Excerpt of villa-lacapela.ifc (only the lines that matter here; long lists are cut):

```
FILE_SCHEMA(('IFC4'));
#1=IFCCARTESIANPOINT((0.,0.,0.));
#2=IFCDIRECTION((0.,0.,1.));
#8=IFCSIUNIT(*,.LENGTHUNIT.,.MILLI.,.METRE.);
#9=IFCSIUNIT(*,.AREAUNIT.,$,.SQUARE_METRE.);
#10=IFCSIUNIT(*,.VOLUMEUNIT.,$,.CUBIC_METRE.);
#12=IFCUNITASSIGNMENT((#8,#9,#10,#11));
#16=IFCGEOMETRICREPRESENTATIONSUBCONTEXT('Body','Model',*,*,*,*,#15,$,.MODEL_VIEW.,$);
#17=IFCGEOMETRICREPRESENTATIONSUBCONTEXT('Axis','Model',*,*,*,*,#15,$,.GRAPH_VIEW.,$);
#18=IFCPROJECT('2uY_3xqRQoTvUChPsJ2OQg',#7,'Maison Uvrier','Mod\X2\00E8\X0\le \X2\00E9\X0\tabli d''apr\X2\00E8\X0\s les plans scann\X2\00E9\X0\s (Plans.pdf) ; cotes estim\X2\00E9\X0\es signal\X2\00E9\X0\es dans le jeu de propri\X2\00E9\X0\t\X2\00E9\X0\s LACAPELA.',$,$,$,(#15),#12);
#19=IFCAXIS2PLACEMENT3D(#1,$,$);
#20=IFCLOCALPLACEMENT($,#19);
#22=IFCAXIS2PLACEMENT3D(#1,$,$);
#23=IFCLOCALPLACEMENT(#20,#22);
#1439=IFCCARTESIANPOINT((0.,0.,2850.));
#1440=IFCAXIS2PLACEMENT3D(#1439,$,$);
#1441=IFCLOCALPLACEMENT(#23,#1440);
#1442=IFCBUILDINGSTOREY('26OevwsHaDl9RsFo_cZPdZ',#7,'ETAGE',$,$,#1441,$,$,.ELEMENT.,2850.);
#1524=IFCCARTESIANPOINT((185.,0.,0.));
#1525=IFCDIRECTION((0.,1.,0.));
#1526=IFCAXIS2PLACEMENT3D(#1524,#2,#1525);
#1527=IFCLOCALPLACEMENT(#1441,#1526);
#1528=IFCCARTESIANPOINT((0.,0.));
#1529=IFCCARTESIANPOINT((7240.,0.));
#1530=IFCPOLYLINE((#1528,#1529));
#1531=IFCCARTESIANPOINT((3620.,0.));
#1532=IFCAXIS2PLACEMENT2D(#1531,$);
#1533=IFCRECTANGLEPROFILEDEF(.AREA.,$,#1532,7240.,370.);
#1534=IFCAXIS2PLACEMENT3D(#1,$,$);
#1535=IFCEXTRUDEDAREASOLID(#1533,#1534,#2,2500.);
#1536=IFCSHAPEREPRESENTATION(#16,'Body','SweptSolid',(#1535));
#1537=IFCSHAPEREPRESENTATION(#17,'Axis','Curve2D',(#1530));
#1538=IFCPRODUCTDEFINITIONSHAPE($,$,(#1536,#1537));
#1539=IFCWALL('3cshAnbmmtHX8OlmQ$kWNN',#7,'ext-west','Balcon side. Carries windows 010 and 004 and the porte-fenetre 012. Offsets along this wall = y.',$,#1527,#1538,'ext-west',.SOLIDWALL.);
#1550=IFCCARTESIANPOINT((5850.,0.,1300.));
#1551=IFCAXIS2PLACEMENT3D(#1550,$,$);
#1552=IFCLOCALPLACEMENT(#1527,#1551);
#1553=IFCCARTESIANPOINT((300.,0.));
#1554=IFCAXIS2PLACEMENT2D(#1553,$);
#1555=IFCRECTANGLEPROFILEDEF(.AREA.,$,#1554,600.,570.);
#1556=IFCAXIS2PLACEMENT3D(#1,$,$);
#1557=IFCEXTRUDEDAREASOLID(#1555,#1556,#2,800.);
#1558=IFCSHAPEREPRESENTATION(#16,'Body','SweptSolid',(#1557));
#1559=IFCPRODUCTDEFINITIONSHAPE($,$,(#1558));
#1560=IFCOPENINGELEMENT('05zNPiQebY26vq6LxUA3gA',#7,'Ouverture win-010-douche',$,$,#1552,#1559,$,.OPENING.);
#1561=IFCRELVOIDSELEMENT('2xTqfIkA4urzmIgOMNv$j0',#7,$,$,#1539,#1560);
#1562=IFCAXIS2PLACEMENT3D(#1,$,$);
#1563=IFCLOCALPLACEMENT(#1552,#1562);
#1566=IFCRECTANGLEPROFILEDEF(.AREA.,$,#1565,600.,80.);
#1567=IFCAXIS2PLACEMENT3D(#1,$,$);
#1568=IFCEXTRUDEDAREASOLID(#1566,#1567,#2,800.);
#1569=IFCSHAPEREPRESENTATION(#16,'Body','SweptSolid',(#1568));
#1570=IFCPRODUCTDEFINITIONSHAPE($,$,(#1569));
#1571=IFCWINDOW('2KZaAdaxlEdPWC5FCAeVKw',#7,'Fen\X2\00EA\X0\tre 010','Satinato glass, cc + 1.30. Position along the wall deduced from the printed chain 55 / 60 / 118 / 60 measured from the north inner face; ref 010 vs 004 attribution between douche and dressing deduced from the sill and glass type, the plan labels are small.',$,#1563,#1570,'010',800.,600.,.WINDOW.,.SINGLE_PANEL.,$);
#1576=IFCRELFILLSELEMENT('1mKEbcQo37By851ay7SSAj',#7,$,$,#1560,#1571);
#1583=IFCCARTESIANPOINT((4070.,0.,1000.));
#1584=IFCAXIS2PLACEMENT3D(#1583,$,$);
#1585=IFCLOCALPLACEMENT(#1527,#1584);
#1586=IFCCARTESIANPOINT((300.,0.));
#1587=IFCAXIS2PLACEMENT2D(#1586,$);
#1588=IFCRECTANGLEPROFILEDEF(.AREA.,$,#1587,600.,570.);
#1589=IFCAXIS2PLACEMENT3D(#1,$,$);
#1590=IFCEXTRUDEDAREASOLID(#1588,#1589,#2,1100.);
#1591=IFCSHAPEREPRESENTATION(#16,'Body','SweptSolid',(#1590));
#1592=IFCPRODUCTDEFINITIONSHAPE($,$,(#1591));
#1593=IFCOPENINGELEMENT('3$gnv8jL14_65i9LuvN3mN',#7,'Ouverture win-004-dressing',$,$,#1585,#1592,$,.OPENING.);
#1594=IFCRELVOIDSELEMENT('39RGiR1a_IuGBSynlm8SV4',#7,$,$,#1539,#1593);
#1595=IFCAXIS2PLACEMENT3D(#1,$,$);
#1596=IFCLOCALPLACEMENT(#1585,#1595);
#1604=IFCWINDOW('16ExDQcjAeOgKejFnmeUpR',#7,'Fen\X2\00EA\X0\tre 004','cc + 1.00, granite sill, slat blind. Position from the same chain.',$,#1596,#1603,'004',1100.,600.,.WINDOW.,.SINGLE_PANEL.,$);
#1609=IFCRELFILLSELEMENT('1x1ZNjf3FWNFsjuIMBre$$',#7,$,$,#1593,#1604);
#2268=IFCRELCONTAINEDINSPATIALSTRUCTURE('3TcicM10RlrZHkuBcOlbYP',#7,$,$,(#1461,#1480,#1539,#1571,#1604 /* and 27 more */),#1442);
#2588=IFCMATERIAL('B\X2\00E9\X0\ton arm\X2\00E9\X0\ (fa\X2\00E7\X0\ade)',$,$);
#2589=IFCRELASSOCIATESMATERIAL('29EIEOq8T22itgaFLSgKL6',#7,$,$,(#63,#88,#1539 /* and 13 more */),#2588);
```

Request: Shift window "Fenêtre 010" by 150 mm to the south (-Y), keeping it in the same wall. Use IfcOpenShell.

```python
import ifcopenshell
import ifcopenshell.api.geometry
import ifcopenshell.util.placement
import ifcopenshell.util.unit

model = ifcopenshell.open("villa-lacapela.ifc")
unit_scale = ifcopenshell.util.unit.calculate_unit_scale(model)

window = model.by_id(1571)
opening = window.FillsVoids[0].RelatingOpeningElement
wall = opening.VoidsElements[0].RelatingBuildingElement

wall_matrix = ifcopenshell.util.placement.get_local_placement(wall.ObjectPlacement)
shift = wall_matrix[:3, 0] * -0.15 / unit_scale
before = ifcopenshell.util.placement.get_local_placement(window.ObjectPlacement)[:3, 3].copy()

# The window is placed relative to its opening, so it follows when the opening moves.
matrix = ifcopenshell.util.placement.get_local_placement(opening.ObjectPlacement)
matrix[:3, 3] += shift
ifcopenshell.api.geometry.edit_object_placement(
    model, product=opening, matrix=matrix, is_si=False, should_transform_children=True
)

after = ifcopenshell.util.placement.get_local_placement(window.ObjectPlacement)[:3, 3]
print("window moved by", (after - before).round(3) + 0.0)

model.write("villa-lacapela_edited.ifc")
```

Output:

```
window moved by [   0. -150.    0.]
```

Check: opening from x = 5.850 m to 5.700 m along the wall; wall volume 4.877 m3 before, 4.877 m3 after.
